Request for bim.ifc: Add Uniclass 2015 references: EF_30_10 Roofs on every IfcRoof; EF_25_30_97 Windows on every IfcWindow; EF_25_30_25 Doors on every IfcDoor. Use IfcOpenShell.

First a look at what the model holds.

```python
import ifcopenshell

model = ifcopenshell.open("bim.ifc")
print(model.schema)
print("classifications:", [c.Name for c in model.by_type("IfcClassification")])
for ifc_class in ("IfcDoor", "IfcRoof", "IfcStair", "IfcWall", "IfcWindow"):
    print(ifc_class, len(model.by_type(ifc_class)))
```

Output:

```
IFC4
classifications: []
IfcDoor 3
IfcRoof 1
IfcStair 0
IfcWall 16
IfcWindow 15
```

```python
import ifcopenshell
import ifcopenshell.api.classification

model = ifcopenshell.open("bim.ifc")

system = ifcopenshell.api.classification.add_classification(model, classification="Uniclass 2015")

codes = {
    "IfcRoof": ("EF_30_10", "Roofs"),
    "IfcWindow": ("EF_25_30_97", "Windows"),
    "IfcDoor": ("EF_25_30_25", "Doors"),
}
for ifc_class, (code, name) in codes.items():
    products = model.by_type(ifc_class)
    ifcopenshell.api.classification.add_reference(
        model, products=products, classification=system, identification=code, name=name
    )
    print(code, len(products))

model.write("bim-out.ifc")
```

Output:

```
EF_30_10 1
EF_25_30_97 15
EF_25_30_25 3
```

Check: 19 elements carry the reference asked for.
